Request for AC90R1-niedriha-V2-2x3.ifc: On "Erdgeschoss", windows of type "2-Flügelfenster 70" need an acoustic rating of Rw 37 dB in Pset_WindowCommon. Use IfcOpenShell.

First a look at what the model holds.

```python
import ifcopenshell
import ifcopenshell.util.element

model = ifcopenshell.open("AC90R1-niedriha-V2-2x3.ifc")
print(model.schema)
storey = next(s for s in model.by_type("IfcBuildingStorey") if s.Name == "Erdgeschoss")
windows = [e for e in ifcopenshell.util.element.get_decomposition(storey) if e.is_a("IfcWindow")]
seen = {}
for e in windows:
    element_type = ifcopenshell.util.element.get_type(e)
    key = (element_type.Name if element_type != e and element_type else None, ifcopenshell.util.element.get_pset(e, "Pset_WindowCommon", "AcousticRating"))
    seen[key] = seen.get(key, 0) + 1
for (name, value), count in sorted(seen.items(), key=str):
    print(count, "x", name, "|", value)
```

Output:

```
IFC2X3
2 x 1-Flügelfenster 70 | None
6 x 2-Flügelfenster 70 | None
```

```python
import ifcopenshell
import ifcopenshell.api.pset
import ifcopenshell.util.element

model = ifcopenshell.open("AC90R1-niedriha-V2-2x3.ifc")

storey = next(s for s in model.by_type("IfcBuildingStorey") if s.Name == "Erdgeschoss")
windows = [e for e in ifcopenshell.util.element.get_decomposition(storey) if e.is_a("IfcWindow")]

count = 0
for e in windows:
    element_type = ifcopenshell.util.element.get_type(e)
    if element_type in (None, e) or element_type.Name != "2-Flügelfenster 70":
        continue
    # add_pset returns the element's existing set when there is one.
    pset = ifcopenshell.api.pset.add_pset(model, product=e, name="Pset_WindowCommon")
    ifcopenshell.api.pset.edit_pset(model, pset=pset, properties={"AcousticRating": "Rw 37 dB"})
    count += 1

print(count, "windows updated")

model.write("AC90R1-niedriha-V2-2x3_rev.ifc")
```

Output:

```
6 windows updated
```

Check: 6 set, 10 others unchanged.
